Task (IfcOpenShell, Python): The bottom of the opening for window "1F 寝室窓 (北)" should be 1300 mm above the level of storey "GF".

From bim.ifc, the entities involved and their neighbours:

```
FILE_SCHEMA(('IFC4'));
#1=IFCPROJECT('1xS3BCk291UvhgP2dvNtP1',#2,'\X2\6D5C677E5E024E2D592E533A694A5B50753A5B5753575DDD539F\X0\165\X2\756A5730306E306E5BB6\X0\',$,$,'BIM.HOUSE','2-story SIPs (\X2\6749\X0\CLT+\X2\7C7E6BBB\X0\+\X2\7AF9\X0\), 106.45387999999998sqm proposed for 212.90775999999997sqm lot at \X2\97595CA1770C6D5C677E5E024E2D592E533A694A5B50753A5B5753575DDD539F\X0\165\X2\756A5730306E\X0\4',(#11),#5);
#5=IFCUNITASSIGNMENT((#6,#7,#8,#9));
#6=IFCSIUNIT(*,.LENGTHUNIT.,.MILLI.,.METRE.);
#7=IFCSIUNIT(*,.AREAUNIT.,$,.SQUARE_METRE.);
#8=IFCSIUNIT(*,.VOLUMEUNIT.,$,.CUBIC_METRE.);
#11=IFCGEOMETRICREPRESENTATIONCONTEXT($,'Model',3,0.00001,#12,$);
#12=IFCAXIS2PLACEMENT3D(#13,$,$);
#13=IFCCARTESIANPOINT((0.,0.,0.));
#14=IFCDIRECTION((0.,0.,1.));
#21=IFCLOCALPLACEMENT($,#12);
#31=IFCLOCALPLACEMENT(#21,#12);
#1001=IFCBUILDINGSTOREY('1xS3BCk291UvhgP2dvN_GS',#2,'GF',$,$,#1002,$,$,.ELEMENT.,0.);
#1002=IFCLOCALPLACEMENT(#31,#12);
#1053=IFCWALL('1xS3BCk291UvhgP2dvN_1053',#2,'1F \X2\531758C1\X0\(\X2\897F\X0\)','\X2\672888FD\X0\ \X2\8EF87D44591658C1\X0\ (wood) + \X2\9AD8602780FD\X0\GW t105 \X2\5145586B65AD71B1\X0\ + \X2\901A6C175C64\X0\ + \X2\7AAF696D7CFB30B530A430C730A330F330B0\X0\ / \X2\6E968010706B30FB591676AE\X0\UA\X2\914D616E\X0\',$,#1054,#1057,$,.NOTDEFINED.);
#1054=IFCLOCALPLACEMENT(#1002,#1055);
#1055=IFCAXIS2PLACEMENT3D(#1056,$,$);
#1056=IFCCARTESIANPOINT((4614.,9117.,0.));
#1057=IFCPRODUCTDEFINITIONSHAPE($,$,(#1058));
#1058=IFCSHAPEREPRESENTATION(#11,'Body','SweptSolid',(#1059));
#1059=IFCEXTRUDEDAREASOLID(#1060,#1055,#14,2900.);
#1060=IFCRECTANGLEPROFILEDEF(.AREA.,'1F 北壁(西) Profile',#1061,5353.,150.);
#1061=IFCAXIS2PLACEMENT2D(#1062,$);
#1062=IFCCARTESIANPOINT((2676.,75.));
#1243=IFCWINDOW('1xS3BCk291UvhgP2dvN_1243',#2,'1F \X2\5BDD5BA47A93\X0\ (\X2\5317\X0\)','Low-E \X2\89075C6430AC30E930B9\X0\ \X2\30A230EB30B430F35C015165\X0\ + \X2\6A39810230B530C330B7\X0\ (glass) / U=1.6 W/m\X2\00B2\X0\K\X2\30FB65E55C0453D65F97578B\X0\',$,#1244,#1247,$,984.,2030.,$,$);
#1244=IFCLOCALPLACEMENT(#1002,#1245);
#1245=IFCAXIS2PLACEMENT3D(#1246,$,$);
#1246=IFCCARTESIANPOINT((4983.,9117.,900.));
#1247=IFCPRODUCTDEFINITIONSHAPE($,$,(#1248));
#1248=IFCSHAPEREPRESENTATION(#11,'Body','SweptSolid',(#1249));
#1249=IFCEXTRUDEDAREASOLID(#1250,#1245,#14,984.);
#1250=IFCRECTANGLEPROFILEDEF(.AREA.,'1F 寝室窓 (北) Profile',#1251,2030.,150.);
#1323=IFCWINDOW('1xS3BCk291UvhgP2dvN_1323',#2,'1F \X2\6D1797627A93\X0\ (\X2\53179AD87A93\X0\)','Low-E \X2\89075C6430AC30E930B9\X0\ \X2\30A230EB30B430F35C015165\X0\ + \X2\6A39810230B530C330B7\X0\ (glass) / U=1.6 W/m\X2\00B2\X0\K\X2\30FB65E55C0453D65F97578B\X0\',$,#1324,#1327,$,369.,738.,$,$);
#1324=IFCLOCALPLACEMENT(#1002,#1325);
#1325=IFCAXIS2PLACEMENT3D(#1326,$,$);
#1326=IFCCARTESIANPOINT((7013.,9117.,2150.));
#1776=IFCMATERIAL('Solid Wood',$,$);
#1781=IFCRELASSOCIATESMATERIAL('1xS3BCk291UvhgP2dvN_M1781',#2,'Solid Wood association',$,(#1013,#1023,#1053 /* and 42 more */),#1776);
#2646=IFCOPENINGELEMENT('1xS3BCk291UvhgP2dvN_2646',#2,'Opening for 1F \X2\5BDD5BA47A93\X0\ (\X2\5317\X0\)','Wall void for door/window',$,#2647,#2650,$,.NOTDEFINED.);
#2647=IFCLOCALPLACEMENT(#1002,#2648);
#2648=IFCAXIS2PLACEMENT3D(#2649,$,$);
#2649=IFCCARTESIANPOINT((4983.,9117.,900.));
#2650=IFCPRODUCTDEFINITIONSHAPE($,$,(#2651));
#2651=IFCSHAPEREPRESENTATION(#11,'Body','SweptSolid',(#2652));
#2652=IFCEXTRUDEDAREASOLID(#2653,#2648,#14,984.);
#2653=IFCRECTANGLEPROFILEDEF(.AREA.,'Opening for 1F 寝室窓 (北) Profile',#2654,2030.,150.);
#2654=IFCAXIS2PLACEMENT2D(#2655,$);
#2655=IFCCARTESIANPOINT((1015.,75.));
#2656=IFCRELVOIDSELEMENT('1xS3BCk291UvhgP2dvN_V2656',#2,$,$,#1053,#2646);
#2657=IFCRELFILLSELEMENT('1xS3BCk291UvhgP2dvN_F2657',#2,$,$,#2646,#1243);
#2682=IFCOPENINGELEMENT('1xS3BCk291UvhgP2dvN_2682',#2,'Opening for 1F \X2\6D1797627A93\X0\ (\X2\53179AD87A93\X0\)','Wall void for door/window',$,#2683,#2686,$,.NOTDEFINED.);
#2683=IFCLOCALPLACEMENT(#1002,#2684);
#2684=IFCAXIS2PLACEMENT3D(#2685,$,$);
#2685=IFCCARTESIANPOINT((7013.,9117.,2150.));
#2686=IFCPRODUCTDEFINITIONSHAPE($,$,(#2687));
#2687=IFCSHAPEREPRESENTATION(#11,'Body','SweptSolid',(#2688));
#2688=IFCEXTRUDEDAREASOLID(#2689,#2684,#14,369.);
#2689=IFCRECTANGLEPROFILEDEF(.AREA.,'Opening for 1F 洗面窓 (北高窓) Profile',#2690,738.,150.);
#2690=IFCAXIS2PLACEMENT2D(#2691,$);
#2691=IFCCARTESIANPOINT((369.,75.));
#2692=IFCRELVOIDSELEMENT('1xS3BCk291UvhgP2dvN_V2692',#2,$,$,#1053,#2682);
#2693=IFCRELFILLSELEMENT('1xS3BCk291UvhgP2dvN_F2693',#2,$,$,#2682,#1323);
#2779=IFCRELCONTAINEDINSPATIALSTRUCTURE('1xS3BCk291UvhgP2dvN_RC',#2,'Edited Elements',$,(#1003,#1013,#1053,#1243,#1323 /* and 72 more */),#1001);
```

```python
import numpy as np
import ifcopenshell
import ifcopenshell.api.geometry
import ifcopenshell.geom
import ifcopenshell.util.element
import ifcopenshell.util.placement
import ifcopenshell.util.shape
import ifcopenshell.util.unit

model = ifcopenshell.open("bim.ifc")
unit_scale = ifcopenshell.util.unit.calculate_unit_scale(model)

window = model.by_id(1243)
opening = window.FillsVoids[0].RelatingOpeningElement
storey = ifcopenshell.util.element.get_container(window, ifc_class="IfcBuildingStorey")
level = ifcopenshell.util.placement.get_local_placement(storey.ObjectPlacement)[2, 3]

# The opening's origin need not be at the sill, so measure its lowest point.
shape = ifcopenshell.geom.create_shape(ifcopenshell.geom.settings(), opening)
bottom = ifcopenshell.util.shape.get_shape_bottom_elevation(shape, shape.geometry) / unit_scale
dz = level + 1.3 / unit_scale - bottom

shift = np.array([0.0, 0.0, dz])
# The window is not placed relative to its opening, so move both.
for product in (opening, window):
    matrix = ifcopenshell.util.placement.get_local_placement(product.ObjectPlacement)
    matrix[:3, 3] += shift
    ifcopenshell.api.geometry.edit_object_placement(model, product=product, matrix=matrix, is_si=False)

print(f"moved by {dz * unit_scale:+.3f} m")

model.write("bim_updated.ifc")
```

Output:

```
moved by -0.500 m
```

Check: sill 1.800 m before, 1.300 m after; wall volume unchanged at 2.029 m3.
